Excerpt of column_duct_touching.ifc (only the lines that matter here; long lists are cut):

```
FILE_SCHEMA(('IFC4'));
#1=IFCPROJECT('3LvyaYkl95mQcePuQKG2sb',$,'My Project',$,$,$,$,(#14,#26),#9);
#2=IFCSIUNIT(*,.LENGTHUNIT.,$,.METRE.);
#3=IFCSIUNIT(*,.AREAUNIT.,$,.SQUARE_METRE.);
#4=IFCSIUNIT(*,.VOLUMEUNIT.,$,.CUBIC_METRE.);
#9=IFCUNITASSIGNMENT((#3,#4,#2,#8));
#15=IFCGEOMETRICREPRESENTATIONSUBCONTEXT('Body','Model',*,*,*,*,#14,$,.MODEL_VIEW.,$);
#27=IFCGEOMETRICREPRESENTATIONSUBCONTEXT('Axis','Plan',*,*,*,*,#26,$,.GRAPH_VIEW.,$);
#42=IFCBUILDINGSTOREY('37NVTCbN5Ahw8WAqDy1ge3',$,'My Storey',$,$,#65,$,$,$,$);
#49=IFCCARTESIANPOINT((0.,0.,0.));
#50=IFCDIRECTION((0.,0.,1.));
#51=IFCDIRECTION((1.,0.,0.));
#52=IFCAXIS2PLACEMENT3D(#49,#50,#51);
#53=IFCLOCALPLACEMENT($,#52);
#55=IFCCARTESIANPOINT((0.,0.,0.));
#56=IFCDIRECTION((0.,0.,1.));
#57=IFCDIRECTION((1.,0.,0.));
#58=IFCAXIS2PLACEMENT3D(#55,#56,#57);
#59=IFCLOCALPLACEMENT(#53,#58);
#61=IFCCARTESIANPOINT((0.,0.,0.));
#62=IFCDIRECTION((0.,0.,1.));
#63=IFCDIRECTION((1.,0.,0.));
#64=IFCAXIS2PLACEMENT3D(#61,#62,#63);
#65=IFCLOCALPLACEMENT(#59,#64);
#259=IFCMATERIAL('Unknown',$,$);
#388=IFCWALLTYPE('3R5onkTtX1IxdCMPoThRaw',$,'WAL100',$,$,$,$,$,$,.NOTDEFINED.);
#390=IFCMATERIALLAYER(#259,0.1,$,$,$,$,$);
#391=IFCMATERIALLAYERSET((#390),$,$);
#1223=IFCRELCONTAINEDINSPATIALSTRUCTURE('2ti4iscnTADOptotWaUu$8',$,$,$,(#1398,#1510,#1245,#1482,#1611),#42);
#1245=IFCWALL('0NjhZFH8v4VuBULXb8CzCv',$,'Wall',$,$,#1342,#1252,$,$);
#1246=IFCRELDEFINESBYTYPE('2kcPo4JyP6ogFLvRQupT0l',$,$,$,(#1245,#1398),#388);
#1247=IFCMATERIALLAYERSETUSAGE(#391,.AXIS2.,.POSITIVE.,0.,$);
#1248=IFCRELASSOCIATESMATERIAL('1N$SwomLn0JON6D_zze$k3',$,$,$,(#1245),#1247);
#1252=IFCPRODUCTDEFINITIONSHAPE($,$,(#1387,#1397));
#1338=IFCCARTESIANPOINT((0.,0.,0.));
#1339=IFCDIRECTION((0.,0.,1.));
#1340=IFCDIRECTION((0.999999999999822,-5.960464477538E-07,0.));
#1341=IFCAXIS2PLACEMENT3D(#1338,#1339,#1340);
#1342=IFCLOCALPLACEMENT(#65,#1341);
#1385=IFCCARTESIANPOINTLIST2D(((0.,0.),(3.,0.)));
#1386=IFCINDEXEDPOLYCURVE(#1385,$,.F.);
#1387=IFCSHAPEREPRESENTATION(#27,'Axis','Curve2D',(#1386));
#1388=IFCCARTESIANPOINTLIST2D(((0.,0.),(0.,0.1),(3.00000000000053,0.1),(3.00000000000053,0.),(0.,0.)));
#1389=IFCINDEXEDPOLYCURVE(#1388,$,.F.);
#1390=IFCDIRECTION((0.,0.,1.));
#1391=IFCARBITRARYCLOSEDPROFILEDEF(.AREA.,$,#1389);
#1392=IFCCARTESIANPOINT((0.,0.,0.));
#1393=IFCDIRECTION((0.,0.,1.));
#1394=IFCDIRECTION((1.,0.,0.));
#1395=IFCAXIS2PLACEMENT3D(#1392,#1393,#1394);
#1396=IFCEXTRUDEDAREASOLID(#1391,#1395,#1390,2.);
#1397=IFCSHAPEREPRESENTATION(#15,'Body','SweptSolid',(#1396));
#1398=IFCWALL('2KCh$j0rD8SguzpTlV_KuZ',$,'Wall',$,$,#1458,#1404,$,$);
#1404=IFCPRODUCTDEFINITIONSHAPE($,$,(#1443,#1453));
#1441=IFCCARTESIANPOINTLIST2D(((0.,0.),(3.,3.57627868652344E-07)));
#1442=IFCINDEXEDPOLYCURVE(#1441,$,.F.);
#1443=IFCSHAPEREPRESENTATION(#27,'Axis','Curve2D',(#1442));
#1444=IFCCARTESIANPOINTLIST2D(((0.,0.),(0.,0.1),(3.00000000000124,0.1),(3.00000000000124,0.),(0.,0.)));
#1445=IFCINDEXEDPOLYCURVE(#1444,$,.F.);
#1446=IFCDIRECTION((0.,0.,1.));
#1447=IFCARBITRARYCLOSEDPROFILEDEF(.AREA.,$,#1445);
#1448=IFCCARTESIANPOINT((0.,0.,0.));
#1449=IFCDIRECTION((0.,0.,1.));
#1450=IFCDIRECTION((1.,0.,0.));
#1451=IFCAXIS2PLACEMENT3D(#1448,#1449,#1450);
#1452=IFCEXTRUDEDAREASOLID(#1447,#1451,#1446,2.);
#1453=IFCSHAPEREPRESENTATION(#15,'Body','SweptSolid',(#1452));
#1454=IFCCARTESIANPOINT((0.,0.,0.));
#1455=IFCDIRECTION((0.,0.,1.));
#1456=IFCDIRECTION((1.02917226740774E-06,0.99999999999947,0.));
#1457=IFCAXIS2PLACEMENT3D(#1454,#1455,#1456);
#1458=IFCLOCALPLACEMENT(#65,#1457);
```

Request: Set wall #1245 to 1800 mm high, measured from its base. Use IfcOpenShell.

```python
import ifcopenshell
import ifcopenshell.geom
import ifcopenshell.util.representation
import ifcopenshell.util.shape

model = ifcopenshell.open("column_duct_touching.ifc")
settings = ifcopenshell.geom.settings()


def volume(element):
    """Net volume in cubic metres, openings subtracted."""
    shape = ifcopenshell.geom.create_shape(settings, element)
    return ifcopenshell.util.shape.get_volume(shape.geometry)


wall = model.by_guid("0NjhZFH8v4VuBULXb8CzCv")
before = volume(wall)

body = ifcopenshell.util.representation.get_representation(wall, "Model", "Body")
solid = body.Items[0]
old_height = solid.Depth
solid.Depth = 1.8
after = volume(wall)

print(f"height {old_height:g} -> {solid.Depth:g}, volume {before:.3f} -> {after:.3f} m3")

model.write("column_duct_touching_edited.ifc")
```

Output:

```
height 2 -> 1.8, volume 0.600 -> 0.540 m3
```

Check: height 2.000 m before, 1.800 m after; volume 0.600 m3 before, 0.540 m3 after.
